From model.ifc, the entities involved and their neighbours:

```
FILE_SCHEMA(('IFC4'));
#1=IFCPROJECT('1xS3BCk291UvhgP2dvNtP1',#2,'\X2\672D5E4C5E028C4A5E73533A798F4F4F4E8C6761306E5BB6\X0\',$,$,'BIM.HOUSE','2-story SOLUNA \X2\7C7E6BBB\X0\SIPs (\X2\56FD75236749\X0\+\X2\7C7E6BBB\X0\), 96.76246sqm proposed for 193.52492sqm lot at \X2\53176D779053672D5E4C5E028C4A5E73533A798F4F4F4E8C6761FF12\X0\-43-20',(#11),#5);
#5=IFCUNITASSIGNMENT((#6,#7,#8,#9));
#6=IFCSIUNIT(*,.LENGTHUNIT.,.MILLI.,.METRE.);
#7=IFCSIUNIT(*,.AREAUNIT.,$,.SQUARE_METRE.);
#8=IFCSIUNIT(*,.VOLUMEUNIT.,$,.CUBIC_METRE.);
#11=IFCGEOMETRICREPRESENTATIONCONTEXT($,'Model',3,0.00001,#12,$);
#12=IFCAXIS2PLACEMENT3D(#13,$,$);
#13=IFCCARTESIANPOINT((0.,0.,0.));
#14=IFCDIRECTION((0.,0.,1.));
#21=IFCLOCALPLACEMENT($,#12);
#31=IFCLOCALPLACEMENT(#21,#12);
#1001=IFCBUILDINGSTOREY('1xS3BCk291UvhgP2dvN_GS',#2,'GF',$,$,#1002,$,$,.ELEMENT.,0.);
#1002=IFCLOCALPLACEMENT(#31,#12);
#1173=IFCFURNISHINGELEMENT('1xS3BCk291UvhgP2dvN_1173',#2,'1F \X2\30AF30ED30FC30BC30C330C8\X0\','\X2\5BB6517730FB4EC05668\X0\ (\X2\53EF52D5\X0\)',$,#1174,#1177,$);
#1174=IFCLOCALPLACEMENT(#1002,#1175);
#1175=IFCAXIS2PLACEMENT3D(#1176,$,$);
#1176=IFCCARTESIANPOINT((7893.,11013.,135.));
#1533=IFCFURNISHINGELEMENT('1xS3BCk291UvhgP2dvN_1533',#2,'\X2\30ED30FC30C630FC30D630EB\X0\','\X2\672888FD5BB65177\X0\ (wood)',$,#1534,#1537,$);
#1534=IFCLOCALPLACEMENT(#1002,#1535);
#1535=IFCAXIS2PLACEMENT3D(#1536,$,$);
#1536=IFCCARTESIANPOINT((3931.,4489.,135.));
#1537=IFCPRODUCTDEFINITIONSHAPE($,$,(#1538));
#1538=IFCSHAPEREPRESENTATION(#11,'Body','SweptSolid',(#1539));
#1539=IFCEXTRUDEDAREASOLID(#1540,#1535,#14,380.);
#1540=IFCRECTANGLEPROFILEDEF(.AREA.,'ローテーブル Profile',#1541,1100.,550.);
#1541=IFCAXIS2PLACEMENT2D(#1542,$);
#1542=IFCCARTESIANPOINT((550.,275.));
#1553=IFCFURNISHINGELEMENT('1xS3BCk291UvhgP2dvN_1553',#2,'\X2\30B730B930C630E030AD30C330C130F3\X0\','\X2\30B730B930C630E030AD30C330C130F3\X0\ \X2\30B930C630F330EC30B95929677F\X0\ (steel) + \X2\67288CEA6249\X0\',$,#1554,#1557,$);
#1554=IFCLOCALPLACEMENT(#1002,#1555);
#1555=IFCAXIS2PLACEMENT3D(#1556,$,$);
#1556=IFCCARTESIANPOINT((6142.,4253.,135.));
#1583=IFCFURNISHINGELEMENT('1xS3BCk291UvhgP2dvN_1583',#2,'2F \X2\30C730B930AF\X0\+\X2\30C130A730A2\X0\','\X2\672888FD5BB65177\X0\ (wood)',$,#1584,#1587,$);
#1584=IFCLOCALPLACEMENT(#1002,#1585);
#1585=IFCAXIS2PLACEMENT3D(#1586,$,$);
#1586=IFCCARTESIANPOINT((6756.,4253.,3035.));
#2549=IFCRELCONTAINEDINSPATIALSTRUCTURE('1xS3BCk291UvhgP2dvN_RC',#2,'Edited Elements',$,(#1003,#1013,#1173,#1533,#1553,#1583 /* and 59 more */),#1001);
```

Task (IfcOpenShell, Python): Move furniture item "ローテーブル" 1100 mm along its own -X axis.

```python
import ifcopenshell
import ifcopenshell.api.geometry
import ifcopenshell.util.placement

model = ifcopenshell.open("model.ifc")

item = model.by_guid("1xS3BCk291UvhgP2dvN_1533")
matrix = ifcopenshell.util.placement.get_local_placement(item.ObjectPlacement)
matrix[:3, 3] -= matrix[:3, 0] * 1100.0
ifcopenshell.api.geometry.edit_object_placement(model, product=item, matrix=matrix, is_si=False)

print(ifcopenshell.util.placement.get_local_placement(item.ObjectPlacement).round(3) + 0.0)

model.write("model_edited.ifc")
```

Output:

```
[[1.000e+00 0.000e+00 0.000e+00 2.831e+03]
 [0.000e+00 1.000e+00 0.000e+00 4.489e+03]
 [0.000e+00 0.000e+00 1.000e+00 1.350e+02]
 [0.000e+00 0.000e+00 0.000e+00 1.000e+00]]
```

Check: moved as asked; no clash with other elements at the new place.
